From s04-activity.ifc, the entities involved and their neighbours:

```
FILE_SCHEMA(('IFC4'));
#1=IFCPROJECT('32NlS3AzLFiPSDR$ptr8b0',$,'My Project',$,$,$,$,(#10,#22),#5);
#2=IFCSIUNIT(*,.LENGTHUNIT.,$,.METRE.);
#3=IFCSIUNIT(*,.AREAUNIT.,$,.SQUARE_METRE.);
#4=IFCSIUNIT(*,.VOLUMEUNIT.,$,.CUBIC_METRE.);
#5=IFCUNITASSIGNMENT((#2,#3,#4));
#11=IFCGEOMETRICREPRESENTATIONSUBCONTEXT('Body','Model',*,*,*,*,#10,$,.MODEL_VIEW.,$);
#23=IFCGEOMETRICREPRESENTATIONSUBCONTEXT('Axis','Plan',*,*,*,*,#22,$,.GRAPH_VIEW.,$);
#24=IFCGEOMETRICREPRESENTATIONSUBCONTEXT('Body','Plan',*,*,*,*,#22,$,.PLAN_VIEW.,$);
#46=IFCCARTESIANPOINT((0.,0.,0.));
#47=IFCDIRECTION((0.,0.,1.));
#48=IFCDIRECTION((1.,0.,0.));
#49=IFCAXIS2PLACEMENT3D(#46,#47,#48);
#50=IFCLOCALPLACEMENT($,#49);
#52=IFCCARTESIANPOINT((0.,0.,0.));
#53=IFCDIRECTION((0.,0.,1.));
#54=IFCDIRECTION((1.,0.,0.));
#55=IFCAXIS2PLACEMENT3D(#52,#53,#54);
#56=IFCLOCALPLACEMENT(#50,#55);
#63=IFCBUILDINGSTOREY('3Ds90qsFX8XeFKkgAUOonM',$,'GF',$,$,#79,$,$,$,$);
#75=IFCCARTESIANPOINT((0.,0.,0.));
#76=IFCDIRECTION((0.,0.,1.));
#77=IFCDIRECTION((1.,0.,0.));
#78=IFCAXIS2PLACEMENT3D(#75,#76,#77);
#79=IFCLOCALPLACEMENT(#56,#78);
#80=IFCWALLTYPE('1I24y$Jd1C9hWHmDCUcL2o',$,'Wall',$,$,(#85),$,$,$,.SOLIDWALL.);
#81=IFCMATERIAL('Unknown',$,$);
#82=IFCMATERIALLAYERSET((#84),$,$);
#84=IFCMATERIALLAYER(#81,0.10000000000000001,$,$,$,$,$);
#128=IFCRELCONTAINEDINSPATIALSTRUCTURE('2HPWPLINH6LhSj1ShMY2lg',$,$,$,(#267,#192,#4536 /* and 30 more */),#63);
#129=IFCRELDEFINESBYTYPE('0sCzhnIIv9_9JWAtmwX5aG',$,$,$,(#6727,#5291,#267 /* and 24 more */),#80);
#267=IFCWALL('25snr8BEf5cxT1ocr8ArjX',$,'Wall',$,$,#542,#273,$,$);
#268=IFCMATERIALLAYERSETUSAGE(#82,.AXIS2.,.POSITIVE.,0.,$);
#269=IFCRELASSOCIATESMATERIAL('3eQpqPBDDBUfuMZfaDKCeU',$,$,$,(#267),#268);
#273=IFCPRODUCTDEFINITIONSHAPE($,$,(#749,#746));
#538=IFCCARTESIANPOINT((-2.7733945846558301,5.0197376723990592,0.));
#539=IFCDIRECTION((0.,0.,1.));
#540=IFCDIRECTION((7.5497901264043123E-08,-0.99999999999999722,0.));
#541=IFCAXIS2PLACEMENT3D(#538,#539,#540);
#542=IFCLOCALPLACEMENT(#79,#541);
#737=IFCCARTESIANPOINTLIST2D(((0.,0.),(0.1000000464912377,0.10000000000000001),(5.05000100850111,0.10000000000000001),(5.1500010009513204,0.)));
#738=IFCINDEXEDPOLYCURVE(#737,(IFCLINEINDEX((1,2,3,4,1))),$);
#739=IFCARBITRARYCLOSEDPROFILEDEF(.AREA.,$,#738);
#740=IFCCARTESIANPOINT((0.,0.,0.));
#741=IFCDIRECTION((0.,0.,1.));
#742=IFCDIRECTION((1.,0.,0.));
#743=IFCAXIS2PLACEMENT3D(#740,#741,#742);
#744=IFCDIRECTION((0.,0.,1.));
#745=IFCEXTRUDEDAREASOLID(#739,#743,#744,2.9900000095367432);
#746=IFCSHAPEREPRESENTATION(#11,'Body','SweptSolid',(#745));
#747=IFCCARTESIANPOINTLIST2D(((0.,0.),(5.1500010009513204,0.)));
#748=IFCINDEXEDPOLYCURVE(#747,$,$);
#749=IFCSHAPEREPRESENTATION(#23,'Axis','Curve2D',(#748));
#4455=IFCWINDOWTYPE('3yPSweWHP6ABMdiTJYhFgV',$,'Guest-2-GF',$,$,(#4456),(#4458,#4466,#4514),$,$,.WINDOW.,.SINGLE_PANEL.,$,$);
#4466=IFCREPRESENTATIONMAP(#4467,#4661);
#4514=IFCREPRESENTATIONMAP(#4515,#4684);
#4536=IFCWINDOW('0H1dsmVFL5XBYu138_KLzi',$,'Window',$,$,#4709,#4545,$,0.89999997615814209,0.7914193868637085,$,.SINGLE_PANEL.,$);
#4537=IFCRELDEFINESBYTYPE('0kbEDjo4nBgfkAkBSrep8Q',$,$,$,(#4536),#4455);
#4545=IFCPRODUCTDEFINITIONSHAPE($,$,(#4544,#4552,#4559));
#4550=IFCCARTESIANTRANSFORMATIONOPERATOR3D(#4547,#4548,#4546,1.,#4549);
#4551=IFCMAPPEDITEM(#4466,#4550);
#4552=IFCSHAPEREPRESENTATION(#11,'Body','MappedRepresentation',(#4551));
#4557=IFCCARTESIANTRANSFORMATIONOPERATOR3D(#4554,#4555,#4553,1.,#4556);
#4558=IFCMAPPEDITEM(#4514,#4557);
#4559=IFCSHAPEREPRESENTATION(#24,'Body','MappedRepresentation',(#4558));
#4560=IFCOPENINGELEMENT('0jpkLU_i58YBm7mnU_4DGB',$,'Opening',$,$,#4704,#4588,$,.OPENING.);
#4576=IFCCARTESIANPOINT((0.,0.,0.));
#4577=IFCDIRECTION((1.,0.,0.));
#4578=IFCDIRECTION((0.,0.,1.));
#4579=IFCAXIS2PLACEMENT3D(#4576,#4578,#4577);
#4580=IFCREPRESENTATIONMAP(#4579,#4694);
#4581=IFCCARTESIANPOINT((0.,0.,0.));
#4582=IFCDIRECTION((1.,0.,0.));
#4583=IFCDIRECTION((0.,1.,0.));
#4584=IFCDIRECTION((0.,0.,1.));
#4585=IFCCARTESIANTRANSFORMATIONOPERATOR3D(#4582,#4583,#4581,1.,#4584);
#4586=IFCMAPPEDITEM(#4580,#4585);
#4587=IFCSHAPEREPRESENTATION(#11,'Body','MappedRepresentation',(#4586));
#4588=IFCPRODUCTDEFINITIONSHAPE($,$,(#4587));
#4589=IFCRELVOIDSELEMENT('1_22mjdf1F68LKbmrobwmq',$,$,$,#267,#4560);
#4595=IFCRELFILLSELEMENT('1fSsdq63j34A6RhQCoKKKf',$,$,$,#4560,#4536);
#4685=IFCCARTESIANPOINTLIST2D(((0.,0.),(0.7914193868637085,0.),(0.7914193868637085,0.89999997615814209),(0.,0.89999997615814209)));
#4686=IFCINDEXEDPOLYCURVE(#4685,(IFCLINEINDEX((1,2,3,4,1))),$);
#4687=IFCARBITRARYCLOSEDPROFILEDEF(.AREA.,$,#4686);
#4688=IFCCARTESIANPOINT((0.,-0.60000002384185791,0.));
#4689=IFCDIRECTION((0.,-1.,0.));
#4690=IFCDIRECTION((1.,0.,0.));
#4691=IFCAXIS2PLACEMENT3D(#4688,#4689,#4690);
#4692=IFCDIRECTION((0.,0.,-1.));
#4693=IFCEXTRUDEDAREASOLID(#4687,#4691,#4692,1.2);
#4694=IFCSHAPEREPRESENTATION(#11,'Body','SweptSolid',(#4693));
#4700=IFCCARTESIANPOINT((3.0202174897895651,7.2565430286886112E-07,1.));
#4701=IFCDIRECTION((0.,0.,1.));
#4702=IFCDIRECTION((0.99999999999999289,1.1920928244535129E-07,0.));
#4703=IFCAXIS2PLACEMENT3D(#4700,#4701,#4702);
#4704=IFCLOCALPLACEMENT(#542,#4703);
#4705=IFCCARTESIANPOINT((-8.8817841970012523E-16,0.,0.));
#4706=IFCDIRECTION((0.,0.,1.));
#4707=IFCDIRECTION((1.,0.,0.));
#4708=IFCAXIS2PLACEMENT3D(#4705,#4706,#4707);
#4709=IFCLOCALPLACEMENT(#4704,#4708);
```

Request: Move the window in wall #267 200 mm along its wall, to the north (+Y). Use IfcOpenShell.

```python
import ifcopenshell
import ifcopenshell.api.geometry
import ifcopenshell.util.placement
import ifcopenshell.util.unit

model = ifcopenshell.open("s04-activity.ifc")
unit_scale = ifcopenshell.util.unit.calculate_unit_scale(model)

window = model.by_guid("0H1dsmVFL5XBYu138_KLzi")
opening = window.FillsVoids[0].RelatingOpeningElement
wall = opening.VoidsElements[0].RelatingBuildingElement

wall_matrix = ifcopenshell.util.placement.get_local_placement(wall.ObjectPlacement)
shift = wall_matrix[:3, 0] * -0.2 / unit_scale
before = ifcopenshell.util.placement.get_local_placement(window.ObjectPlacement)[:3, 3].copy()

# The window is placed relative to its opening, so it follows when the opening moves.
matrix = ifcopenshell.util.placement.get_local_placement(opening.ObjectPlacement)
matrix[:3, 3] += shift
ifcopenshell.api.geometry.edit_object_placement(
    model, product=opening, matrix=matrix, is_si=False, should_transform_children=True
)

after = ifcopenshell.util.placement.get_local_placement(window.ObjectPlacement)[:3, 3]
print("window moved by", (after - before).round(3) + 0.0)

model.write("s04-activity-out.ifc")
```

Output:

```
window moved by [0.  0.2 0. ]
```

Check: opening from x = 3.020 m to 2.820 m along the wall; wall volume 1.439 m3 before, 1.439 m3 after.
